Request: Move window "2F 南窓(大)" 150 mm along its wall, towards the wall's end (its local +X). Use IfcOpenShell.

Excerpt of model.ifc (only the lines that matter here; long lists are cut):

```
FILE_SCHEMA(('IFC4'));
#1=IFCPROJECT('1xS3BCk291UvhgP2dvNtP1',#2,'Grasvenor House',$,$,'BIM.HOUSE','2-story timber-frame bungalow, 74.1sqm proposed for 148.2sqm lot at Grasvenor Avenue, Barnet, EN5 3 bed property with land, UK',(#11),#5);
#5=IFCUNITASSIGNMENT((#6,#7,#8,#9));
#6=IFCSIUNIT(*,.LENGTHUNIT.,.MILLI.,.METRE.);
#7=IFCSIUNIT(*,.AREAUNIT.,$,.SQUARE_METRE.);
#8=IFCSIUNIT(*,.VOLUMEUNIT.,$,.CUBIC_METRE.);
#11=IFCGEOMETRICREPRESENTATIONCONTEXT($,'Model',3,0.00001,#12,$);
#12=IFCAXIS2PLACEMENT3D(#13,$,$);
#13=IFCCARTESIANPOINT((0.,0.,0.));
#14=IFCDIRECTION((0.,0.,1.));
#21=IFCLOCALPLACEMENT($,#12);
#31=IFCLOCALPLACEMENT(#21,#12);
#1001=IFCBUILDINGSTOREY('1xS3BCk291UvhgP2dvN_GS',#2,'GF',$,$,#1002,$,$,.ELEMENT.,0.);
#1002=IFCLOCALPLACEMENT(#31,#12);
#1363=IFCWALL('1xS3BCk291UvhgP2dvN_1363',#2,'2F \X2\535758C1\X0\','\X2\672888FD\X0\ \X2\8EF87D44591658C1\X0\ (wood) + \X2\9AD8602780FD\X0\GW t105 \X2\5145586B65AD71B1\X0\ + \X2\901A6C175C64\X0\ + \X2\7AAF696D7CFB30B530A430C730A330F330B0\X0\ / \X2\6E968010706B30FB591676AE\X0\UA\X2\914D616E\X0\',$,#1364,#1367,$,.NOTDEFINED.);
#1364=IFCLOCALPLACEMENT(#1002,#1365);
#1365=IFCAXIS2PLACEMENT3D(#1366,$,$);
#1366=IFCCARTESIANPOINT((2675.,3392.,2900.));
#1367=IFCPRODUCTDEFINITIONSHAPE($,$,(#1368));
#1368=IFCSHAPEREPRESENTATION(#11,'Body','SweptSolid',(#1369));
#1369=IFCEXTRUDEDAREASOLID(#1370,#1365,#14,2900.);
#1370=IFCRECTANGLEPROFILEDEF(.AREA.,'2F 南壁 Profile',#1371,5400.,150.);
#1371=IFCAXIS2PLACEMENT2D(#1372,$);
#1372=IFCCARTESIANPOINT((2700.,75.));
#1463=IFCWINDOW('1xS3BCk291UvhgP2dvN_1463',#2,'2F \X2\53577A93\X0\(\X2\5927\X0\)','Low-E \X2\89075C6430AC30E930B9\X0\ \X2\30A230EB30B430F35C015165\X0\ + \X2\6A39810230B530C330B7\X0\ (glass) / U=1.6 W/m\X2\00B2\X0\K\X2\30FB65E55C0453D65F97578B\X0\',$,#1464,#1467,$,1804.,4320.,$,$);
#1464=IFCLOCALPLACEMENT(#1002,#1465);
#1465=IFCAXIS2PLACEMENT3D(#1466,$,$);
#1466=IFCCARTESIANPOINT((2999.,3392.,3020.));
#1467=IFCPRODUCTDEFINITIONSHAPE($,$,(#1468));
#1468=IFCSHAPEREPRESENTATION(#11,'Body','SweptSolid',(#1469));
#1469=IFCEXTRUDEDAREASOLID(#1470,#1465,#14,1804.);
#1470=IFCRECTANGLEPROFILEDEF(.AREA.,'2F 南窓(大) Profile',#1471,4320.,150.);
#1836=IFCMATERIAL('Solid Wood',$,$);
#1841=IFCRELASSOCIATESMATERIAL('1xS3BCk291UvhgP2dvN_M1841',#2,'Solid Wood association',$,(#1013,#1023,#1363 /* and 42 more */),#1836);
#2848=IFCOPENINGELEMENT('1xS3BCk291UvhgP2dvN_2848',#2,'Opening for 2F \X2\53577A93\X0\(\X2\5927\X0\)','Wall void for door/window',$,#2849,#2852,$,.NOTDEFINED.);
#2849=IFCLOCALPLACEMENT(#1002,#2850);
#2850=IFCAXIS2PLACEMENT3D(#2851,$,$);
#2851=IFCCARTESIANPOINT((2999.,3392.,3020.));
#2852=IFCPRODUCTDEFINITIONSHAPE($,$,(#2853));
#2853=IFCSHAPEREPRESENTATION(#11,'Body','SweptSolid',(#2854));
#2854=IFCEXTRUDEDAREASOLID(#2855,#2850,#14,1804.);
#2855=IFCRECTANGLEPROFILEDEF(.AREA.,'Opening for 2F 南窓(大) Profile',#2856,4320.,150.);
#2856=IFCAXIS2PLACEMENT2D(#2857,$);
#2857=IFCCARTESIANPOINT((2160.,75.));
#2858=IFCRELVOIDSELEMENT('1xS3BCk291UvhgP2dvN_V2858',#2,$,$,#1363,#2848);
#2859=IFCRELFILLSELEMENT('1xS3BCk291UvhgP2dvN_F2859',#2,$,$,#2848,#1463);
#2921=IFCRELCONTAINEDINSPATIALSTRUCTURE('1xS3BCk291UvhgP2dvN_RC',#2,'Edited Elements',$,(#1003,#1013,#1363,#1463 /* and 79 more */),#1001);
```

```python
import ifcopenshell
import ifcopenshell.api.geometry
import ifcopenshell.util.placement

model = ifcopenshell.open("model.ifc")

window = model.by_guid("1xS3BCk291UvhgP2dvN_1463")
opening = window.FillsVoids[0].RelatingOpeningElement
wall = opening.VoidsElements[0].RelatingBuildingElement

wall_matrix = ifcopenshell.util.placement.get_local_placement(wall.ObjectPlacement)
shift = wall_matrix[:3, 0] * 150.0
before = ifcopenshell.util.placement.get_local_placement(window.ObjectPlacement)[:3, 3].copy()

# The window is not placed relative to its opening, so move both.
for product in (opening, window):
    matrix = ifcopenshell.util.placement.get_local_placement(product.ObjectPlacement)
    matrix[:3, 3] += shift
    ifcopenshell.api.geometry.edit_object_placement(model, product=product, matrix=matrix, is_si=False)

after = ifcopenshell.util.placement.get_local_placement(window.ObjectPlacement)[:3, 3]
print("window moved by", (after - before).round(3) + 0.0)

model.write("model_edited.ifc")
```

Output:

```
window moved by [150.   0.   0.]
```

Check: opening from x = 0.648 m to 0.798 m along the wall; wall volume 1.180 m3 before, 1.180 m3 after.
